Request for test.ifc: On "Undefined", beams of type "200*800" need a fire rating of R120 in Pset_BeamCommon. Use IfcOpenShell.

First a look at what the model holds.

```python
import ifcopenshell
import ifcopenshell.util.element

model = ifcopenshell.open("test.ifc")
print(model.schema)
storey = next(s for s in model.by_type("IfcBuildingStorey") if s.Name == "Undefined")
beams = [e for e in ifcopenshell.util.element.get_decomposition(storey) if e.is_a("IfcBeam")]
seen = {}
for e in beams:
    element_type = ifcopenshell.util.element.get_type(e)
    key = (element_type.Name if element_type != e and element_type else None, ifcopenshell.util.element.get_pset(e, "Pset_BeamCommon", "FireRating"))
    seen[key] = seen.get(key, 0) + 1
for (name, value), count in sorted(seen.items(), key=str):
    print(count, "x", name, "|", value)
```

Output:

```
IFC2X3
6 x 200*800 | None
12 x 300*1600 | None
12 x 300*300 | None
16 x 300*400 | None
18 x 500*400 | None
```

```python
import ifcopenshell
import ifcopenshell.api.pset
import ifcopenshell.util.element

model = ifcopenshell.open("test.ifc")

storey = next(s for s in model.by_type("IfcBuildingStorey") if s.Name == "Undefined")
beams = [e for e in ifcopenshell.util.element.get_decomposition(storey) if e.is_a("IfcBeam")]

count = 0
for e in beams:
    element_type = ifcopenshell.util.element.get_type(e)
    if element_type in (None, e) or element_type.Name != "200*800":
        continue
    found = ifcopenshell.util.element.get_pset(e, "Pset_BeamCommon", should_inherit=False)
    if found:
        pset = model.by_id(found["id"])
        if len(ifcopenshell.util.element.get_elements_by_pset(pset)) > 1:
            pset = ifcopenshell.api.pset.unshare_pset(model, products=[e], pset=pset)[0]
    else:
        pset = ifcopenshell.api.pset.add_pset(model, product=e, name="Pset_BeamCommon")
    ifcopenshell.api.pset.edit_pset(model, pset=pset, properties={"FireRating": "R120"})
    count += 1

print(count, "beams updated")

model.write("test_edited.ifc")
```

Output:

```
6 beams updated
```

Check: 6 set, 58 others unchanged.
